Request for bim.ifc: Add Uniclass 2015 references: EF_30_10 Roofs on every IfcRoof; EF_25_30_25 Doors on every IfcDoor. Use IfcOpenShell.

First a look at what the model holds.

```python
import ifcopenshell

model = ifcopenshell.open("bim.ifc")
print(model.schema)
print("classifications:", [c.Name for c in model.by_type("IfcClassification")])
for ifc_class in ("IfcDoor", "IfcRoof", "IfcStair", "IfcWall", "IfcWindow"):
    print(ifc_class, len(model.by_type(ifc_class)))
```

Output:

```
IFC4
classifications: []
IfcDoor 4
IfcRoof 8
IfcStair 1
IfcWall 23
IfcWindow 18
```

```python
import ifcopenshell
import ifcopenshell.api.classification

model = ifcopenshell.open("bim.ifc")

system = ifcopenshell.api.classification.add_classification(model, classification="Uniclass 2015")

codes = {
    "IfcRoof": ("EF_30_10", "Roofs"),
    "IfcDoor": ("EF_25_30_25", "Doors"),
}
for ifc_class, (code, name) in codes.items():
    products = model.by_type(ifc_class)
    ifcopenshell.api.classification.add_reference(
        model, products=products, classification=system, identification=code, name=name
    )
    print(code, len(products))

model.write("bim_rev.ifc")
```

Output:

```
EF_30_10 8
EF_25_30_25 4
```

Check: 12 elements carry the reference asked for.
